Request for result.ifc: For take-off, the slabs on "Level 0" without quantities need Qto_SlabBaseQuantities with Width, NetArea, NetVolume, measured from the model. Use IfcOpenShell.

First a look at what the model holds.

```python
import ifcopenshell
import ifcopenshell.util.element
import ifcopenshell.util.unit

model = ifcopenshell.open("result.ifc")
print(model.schema)
for unit_type in ("LENGTHUNIT", "AREAUNIT", "VOLUMEUNIT"):
    print(unit_type, ifcopenshell.util.unit.calculate_unit_scale(model, unit_type))
storey = next(s for s in model.by_type("IfcBuildingStorey") if s.Name == "Level 0")
slabs = [e for e in ifcopenshell.util.element.get_decomposition(storey) if e.is_a("IfcSlab")]
for e in sorted(slabs, key=lambda e: e.id()):
    print(e.id(), e.is_a(), e.Name, list(ifcopenshell.util.element.get_psets(e, qtos_only=True)), sep=" | ")
```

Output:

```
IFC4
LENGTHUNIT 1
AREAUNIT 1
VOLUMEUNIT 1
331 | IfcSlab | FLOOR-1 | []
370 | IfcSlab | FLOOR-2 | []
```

```python
import ifcopenshell
import ifcopenshell.api.pset
import ifcopenshell.geom
import ifcopenshell.util.element
import ifcopenshell.util.shape
import ifcopenshell.util.unit

model = ifcopenshell.open("result.ifc")
unit_scale = ifcopenshell.util.unit.calculate_unit_scale(model)
area_scale = ifcopenshell.util.unit.calculate_unit_scale(model, "AREAUNIT")
volume_scale = ifcopenshell.util.unit.calculate_unit_scale(model, "VOLUMEUNIT")
settings = ifcopenshell.geom.settings()

storey = next(s for s in model.by_type("IfcBuildingStorey") if s.Name == "Level 0")
slabs = [e for e in ifcopenshell.util.element.get_decomposition(storey) if e.is_a("IfcSlab")]

for e in sorted(slabs, key=lambda e: e.id()):
    if ifcopenshell.util.element.get_psets(e, qtos_only=True, should_inherit=False):
        continue
    # Geometry comes back in metres, in the element's own axes.
    shape = ifcopenshell.geom.create_shape(settings, e)
    values = {
        "Width": ifcopenshell.util.shape.get_z(shape.geometry) / unit_scale,
        "NetArea": ifcopenshell.util.shape.get_footprint_area(shape.geometry) / area_scale,
        "NetVolume": ifcopenshell.util.shape.get_volume(shape.geometry) / volume_scale,
    }
    qto = ifcopenshell.api.pset.add_qto(model, product=e, name="Qto_SlabBaseQuantities")
    ifcopenshell.api.pset.edit_qto(model, qto=qto, properties=values)
    print(e.id(), {k: round(v, 3) for k, v in values.items()})

model.write("result_rev.ifc")
```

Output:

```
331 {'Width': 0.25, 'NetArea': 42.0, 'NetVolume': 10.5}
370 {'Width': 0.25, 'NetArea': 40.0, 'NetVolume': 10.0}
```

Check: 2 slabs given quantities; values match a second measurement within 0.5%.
